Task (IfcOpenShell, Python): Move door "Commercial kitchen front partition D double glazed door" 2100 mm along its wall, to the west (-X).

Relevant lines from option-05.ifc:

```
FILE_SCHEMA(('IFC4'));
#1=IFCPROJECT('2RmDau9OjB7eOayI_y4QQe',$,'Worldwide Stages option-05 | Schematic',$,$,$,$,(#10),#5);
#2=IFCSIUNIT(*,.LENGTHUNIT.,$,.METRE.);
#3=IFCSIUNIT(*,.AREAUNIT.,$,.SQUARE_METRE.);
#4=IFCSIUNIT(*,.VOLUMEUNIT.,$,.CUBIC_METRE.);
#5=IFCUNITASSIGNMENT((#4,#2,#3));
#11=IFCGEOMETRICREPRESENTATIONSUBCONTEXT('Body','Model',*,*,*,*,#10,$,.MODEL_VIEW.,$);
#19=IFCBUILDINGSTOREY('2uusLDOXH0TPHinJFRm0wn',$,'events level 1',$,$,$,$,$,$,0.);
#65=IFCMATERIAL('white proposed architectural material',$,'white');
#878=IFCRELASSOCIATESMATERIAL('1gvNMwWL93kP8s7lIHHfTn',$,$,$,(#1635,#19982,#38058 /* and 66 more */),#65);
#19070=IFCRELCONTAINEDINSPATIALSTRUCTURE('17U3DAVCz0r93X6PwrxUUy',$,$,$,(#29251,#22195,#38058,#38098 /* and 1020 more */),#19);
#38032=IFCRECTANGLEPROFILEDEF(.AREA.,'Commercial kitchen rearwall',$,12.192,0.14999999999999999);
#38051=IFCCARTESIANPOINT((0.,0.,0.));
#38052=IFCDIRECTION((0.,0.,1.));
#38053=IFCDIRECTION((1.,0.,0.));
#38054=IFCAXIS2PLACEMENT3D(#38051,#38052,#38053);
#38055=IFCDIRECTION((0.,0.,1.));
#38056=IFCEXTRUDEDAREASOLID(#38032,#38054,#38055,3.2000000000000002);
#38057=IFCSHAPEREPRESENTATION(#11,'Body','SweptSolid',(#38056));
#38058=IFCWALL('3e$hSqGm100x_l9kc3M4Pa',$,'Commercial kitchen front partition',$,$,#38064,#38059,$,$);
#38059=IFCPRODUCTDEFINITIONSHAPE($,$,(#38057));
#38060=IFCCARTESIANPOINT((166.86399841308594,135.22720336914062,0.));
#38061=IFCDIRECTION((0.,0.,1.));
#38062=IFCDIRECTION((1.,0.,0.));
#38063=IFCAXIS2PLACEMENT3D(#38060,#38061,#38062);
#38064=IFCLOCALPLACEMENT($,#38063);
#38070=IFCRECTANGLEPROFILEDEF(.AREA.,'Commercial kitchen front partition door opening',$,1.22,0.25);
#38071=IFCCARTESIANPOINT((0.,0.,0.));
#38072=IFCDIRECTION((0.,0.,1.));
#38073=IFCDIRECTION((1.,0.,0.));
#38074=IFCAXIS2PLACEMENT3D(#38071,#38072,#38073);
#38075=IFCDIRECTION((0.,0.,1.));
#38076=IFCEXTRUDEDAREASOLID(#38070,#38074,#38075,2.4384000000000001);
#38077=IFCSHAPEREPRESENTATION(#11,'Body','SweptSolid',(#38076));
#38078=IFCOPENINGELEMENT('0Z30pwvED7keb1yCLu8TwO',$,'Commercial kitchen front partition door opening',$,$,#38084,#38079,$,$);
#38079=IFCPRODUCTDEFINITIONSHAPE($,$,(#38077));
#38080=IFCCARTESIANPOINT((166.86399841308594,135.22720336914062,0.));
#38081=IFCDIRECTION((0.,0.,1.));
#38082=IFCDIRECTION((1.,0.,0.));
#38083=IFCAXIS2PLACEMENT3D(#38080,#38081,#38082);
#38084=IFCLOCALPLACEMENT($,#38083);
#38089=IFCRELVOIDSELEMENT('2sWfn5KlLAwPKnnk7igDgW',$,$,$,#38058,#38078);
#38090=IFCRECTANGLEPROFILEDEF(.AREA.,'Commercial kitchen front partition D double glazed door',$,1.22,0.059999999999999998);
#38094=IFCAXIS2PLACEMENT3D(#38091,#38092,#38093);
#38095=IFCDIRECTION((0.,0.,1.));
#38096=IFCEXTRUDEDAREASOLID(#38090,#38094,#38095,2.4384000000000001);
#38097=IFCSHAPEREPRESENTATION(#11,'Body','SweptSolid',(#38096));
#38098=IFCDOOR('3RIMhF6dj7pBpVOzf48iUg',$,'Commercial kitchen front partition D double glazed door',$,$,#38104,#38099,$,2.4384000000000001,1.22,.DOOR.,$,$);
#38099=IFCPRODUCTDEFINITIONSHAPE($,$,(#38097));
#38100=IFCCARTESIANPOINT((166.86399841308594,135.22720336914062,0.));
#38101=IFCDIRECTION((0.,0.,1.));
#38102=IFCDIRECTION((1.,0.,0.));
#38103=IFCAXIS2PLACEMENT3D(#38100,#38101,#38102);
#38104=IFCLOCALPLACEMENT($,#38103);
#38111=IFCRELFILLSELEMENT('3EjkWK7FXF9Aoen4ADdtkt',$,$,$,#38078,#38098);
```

```python
import ifcopenshell
import ifcopenshell.api.geometry
import ifcopenshell.util.placement

model = ifcopenshell.open("option-05.ifc")

door = model.by_id(38098)
opening = door.FillsVoids[0].RelatingOpeningElement
wall = opening.VoidsElements[0].RelatingBuildingElement

wall_matrix = ifcopenshell.util.placement.get_local_placement(wall.ObjectPlacement)
shift = wall_matrix[:3, 0] * -2.1
before = ifcopenshell.util.placement.get_local_placement(door.ObjectPlacement)[:3, 3].copy()

# The door is not placed relative to its opening, so move both.
for product in (opening, door):
    matrix = ifcopenshell.util.placement.get_local_placement(product.ObjectPlacement)
    matrix[:3, 3] += shift
    ifcopenshell.api.geometry.edit_object_placement(model, product=product, matrix=matrix, is_si=False)

after = ifcopenshell.util.placement.get_local_placement(door.ObjectPlacement)[:3, 3]
print("door moved by", (after - before).round(3) + 0.0)

model.write("option-05_rev.ifc")
```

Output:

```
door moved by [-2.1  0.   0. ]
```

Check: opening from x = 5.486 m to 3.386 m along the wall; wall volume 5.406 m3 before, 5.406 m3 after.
